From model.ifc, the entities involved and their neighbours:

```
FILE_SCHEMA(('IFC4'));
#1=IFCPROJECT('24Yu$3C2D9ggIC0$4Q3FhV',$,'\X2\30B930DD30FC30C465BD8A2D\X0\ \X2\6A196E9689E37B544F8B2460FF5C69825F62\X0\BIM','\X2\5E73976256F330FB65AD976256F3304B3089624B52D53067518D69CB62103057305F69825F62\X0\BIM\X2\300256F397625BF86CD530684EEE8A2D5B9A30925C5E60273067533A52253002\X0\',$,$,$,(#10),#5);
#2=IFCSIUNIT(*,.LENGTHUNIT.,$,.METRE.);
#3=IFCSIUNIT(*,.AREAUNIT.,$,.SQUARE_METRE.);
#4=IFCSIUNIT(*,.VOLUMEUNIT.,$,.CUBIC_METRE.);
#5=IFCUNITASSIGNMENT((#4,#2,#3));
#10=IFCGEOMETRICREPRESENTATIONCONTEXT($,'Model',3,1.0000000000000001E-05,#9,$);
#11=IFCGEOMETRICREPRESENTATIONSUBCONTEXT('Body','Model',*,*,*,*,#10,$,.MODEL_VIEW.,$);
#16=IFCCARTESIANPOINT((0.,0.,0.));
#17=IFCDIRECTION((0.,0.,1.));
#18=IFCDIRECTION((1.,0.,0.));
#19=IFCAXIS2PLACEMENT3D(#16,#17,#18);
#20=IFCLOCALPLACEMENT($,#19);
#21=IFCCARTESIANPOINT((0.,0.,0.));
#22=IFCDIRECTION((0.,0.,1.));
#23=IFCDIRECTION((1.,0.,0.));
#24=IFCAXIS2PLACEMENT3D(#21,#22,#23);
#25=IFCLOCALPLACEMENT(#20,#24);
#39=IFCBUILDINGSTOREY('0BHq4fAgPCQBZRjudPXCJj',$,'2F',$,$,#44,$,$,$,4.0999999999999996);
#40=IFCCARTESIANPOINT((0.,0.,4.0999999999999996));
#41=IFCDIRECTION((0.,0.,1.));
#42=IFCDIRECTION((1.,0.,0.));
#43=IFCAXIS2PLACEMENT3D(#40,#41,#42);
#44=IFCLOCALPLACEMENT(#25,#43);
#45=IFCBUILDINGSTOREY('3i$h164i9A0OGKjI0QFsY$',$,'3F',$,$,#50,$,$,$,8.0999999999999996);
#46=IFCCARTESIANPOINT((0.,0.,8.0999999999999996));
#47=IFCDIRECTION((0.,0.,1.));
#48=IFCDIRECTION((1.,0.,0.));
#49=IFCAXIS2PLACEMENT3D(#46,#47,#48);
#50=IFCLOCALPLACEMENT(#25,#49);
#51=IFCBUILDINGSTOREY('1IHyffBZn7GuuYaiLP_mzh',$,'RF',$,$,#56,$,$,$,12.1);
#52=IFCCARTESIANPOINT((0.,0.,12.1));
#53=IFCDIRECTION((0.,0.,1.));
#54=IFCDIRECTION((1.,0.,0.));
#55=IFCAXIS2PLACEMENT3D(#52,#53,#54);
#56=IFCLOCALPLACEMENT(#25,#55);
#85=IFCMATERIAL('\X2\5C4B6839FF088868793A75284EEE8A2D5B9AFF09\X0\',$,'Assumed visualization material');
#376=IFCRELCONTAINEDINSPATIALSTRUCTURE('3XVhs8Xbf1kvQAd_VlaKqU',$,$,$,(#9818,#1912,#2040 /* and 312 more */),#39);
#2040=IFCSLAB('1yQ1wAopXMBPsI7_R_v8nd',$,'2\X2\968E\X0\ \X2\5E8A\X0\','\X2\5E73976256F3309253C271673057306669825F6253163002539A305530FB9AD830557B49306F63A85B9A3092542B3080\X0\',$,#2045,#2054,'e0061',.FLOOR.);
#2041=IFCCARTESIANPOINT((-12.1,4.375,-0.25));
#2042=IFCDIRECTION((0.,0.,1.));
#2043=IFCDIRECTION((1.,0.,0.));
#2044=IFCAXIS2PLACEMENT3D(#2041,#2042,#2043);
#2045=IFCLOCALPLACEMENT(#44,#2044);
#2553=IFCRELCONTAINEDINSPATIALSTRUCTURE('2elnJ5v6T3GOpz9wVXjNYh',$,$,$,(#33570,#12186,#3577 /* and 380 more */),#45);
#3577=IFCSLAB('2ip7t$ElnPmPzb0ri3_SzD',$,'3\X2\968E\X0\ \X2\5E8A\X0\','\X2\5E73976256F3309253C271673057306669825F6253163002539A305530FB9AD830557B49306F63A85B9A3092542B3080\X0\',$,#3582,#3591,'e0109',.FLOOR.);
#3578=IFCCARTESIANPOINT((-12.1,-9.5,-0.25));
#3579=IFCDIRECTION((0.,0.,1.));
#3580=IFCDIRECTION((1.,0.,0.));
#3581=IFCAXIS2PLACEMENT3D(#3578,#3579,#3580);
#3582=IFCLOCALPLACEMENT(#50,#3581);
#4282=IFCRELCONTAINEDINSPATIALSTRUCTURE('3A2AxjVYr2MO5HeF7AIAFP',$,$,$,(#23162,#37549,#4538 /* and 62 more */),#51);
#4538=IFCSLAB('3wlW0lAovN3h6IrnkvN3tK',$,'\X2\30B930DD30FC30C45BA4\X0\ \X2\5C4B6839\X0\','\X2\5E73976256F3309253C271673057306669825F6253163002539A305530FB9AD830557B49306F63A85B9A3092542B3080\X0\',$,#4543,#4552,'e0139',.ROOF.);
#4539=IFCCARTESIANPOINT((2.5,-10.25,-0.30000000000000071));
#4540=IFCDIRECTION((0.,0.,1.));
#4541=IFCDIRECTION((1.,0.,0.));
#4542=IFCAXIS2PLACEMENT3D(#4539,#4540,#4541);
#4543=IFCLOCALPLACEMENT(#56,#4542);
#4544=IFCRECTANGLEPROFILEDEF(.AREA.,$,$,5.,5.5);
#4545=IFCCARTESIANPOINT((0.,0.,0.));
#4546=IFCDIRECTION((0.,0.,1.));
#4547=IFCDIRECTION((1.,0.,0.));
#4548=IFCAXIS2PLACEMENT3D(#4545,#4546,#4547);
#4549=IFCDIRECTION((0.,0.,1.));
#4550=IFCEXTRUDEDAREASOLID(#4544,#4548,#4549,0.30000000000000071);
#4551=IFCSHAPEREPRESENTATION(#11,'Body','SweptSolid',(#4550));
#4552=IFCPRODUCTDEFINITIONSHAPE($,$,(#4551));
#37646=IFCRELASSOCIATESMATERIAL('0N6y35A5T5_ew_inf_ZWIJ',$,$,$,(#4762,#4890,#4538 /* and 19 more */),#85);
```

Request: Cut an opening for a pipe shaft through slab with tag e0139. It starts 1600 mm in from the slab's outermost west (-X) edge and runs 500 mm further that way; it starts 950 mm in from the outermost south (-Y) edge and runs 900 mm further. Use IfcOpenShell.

```python
import numpy as np
import ifcopenshell
import ifcopenshell.api.feature
import ifcopenshell.api.geometry
import ifcopenshell.api.root
import ifcopenshell.geom
import ifcopenshell.util.placement
import ifcopenshell.util.representation
import ifcopenshell.util.shape
import ifcopenshell.util.unit

model = ifcopenshell.open("model.ifc")
unit_scale = ifcopenshell.util.unit.calculate_unit_scale(model)
settings = ifcopenshell.geom.settings()


def volume(element):
    """Net volume in cubic metres, openings subtracted."""
    shape = ifcopenshell.geom.create_shape(settings, element)
    return ifcopenshell.util.shape.get_volume(shape.geometry)


slab = model.by_guid("3wlW0lAovN3h6IrnkvN3tK")
before = volume(slab)

# Extent in the slab's own axes, in metres. The edges named are its -X and -Y sides.
slab_shape = ifcopenshell.geom.create_shape(settings, slab)
vertices = ifcopenshell.util.shape.get_vertices(slab_shape.geometry)
x_min, y_min, bottom = vertices.min(axis=0)
top = vertices[:, 2].max()

opening = ifcopenshell.api.root.create_entity(model, ifc_class="IfcOpeningElement", name="Pipe shaft opening", predefined_type="OPENING")
context = ifcopenshell.util.representation.get_context(model, "Model", "Body", "MODEL_VIEW")
width, depth = 0.5, 0.9
outline = [(0.0, 0.0), (width, 0.0), (width, depth), (0.0, depth), (0.0, 0.0)]
# Overshoot both faces by 50 mm so the cut is clean.
shape = ifcopenshell.api.geometry.add_slab_representation(
    model, context=context, depth=top - bottom + 0.1, polyline=outline
)
ifcopenshell.api.geometry.assign_representation(model, product=opening, representation=shape)

matrix = ifcopenshell.util.placement.get_local_placement(slab.ObjectPlacement)
matrix[:, 3] = matrix @ np.append(np.array([x_min + 1.6, y_min + 0.95, bottom - 0.05]) / unit_scale, 1.0)
ifcopenshell.api.geometry.edit_object_placement(model, product=opening, matrix=matrix, is_si=False)
ifcopenshell.api.feature.add_feature(model, feature=opening, element=slab)

after = volume(slab)

print(f"slab volume {before:.3f} -> {after:.3f} m3")

model.write("model_updated.ifc")
```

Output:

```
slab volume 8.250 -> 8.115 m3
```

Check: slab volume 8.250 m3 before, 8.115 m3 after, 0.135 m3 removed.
